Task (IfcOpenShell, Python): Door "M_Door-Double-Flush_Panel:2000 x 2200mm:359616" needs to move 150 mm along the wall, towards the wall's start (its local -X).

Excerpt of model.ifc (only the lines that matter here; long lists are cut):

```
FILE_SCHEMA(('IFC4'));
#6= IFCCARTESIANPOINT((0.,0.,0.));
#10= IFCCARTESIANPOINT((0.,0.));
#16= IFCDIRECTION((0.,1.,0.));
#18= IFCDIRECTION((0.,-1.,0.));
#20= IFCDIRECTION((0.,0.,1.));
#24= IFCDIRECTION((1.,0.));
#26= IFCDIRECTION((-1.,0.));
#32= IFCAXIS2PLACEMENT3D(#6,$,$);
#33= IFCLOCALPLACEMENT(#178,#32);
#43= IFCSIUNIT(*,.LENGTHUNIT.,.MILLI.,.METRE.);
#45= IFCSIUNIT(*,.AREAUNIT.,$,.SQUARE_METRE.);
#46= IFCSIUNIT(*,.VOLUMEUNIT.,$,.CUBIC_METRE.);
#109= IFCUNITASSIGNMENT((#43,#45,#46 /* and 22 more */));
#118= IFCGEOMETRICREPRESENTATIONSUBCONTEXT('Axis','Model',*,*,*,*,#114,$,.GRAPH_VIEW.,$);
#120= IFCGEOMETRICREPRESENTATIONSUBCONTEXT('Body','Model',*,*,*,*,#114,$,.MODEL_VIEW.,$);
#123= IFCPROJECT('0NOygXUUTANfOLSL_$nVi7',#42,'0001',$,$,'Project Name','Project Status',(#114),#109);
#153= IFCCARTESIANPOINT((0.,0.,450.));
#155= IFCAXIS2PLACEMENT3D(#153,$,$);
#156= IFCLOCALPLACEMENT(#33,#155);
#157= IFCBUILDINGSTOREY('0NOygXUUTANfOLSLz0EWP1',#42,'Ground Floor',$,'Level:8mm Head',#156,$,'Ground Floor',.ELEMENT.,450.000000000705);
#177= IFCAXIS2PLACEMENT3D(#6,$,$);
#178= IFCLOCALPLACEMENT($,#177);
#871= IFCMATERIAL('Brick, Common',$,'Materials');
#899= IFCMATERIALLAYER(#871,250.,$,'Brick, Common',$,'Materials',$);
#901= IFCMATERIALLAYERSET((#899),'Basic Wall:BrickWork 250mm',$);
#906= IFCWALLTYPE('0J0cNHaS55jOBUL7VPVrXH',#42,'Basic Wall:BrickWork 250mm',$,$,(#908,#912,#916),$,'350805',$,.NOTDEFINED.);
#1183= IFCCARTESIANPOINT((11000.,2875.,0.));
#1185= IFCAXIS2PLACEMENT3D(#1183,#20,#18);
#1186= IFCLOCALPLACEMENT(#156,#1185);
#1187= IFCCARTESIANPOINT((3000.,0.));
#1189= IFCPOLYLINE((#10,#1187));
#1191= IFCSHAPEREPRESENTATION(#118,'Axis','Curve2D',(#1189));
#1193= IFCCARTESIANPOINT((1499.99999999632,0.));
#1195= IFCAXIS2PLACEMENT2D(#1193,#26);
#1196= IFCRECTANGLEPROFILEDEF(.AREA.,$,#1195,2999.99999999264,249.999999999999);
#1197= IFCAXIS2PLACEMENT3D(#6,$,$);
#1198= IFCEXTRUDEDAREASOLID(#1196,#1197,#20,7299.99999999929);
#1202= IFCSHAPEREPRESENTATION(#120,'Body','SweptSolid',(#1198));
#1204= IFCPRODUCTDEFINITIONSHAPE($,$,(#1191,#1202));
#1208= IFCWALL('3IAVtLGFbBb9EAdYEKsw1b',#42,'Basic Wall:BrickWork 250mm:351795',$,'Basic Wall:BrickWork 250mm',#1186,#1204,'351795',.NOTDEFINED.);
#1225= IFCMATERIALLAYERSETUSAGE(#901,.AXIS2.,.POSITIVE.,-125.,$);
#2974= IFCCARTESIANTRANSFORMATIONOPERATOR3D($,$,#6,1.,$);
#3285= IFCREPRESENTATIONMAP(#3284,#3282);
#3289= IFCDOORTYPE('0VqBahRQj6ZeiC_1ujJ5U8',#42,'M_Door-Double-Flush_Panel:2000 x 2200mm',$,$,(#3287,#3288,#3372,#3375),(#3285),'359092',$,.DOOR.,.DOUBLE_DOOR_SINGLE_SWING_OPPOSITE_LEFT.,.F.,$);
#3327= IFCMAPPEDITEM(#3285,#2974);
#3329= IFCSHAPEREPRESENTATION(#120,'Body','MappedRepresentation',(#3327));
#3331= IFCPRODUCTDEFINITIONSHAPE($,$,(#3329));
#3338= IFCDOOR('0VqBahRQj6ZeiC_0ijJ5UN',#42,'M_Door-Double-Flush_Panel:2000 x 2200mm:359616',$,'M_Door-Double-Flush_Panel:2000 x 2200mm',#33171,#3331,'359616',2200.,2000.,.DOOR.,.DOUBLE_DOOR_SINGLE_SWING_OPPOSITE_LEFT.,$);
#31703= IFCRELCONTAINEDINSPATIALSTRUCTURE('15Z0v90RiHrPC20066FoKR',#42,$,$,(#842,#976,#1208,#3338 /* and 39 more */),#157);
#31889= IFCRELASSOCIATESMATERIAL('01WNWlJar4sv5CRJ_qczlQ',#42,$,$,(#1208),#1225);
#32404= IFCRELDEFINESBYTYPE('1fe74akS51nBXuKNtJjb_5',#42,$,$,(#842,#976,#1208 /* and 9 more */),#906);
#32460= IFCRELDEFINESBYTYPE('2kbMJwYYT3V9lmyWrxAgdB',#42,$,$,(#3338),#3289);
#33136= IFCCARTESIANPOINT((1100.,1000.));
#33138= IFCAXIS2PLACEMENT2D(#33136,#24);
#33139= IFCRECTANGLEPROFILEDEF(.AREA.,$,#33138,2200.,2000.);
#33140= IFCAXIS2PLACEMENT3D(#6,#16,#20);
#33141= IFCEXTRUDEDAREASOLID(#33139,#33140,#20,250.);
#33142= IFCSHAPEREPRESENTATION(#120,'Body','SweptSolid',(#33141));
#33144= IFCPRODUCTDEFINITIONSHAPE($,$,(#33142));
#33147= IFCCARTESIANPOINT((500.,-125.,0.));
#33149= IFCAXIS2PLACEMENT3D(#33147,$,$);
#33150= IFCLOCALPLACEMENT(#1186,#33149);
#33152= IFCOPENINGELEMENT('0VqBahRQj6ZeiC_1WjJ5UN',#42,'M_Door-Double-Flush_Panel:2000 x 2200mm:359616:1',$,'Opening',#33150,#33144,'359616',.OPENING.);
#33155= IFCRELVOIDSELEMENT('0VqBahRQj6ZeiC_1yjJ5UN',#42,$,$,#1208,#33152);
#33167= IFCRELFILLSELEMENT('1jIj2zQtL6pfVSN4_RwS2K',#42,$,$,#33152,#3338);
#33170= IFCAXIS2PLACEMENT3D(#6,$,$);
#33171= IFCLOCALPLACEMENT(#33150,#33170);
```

```python
import ifcopenshell
import ifcopenshell.api.geometry
import ifcopenshell.util.placement

model = ifcopenshell.open("model.ifc")

door = model.by_guid("0VqBahRQj6ZeiC_0ijJ5UN")
opening = door.FillsVoids[0].RelatingOpeningElement
wall = opening.VoidsElements[0].RelatingBuildingElement

wall_matrix = ifcopenshell.util.placement.get_local_placement(wall.ObjectPlacement)
shift = wall_matrix[:3, 0] * -150.0
before = ifcopenshell.util.placement.get_local_placement(door.ObjectPlacement)[:3, 3].copy()

# The door is placed relative to its opening, so it follows when the opening moves.
matrix = ifcopenshell.util.placement.get_local_placement(opening.ObjectPlacement)
matrix[:3, 3] += shift
ifcopenshell.api.geometry.edit_object_placement(
    model, product=opening, matrix=matrix, is_si=False, should_transform_children=True
)

after = ifcopenshell.util.placement.get_local_placement(door.ObjectPlacement)[:3, 3]
print("door moved by", (after - before).round(3) + 0.0)

model.write("model_updated.ifc")
```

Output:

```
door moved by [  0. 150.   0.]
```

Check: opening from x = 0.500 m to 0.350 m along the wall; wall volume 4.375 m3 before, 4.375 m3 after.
